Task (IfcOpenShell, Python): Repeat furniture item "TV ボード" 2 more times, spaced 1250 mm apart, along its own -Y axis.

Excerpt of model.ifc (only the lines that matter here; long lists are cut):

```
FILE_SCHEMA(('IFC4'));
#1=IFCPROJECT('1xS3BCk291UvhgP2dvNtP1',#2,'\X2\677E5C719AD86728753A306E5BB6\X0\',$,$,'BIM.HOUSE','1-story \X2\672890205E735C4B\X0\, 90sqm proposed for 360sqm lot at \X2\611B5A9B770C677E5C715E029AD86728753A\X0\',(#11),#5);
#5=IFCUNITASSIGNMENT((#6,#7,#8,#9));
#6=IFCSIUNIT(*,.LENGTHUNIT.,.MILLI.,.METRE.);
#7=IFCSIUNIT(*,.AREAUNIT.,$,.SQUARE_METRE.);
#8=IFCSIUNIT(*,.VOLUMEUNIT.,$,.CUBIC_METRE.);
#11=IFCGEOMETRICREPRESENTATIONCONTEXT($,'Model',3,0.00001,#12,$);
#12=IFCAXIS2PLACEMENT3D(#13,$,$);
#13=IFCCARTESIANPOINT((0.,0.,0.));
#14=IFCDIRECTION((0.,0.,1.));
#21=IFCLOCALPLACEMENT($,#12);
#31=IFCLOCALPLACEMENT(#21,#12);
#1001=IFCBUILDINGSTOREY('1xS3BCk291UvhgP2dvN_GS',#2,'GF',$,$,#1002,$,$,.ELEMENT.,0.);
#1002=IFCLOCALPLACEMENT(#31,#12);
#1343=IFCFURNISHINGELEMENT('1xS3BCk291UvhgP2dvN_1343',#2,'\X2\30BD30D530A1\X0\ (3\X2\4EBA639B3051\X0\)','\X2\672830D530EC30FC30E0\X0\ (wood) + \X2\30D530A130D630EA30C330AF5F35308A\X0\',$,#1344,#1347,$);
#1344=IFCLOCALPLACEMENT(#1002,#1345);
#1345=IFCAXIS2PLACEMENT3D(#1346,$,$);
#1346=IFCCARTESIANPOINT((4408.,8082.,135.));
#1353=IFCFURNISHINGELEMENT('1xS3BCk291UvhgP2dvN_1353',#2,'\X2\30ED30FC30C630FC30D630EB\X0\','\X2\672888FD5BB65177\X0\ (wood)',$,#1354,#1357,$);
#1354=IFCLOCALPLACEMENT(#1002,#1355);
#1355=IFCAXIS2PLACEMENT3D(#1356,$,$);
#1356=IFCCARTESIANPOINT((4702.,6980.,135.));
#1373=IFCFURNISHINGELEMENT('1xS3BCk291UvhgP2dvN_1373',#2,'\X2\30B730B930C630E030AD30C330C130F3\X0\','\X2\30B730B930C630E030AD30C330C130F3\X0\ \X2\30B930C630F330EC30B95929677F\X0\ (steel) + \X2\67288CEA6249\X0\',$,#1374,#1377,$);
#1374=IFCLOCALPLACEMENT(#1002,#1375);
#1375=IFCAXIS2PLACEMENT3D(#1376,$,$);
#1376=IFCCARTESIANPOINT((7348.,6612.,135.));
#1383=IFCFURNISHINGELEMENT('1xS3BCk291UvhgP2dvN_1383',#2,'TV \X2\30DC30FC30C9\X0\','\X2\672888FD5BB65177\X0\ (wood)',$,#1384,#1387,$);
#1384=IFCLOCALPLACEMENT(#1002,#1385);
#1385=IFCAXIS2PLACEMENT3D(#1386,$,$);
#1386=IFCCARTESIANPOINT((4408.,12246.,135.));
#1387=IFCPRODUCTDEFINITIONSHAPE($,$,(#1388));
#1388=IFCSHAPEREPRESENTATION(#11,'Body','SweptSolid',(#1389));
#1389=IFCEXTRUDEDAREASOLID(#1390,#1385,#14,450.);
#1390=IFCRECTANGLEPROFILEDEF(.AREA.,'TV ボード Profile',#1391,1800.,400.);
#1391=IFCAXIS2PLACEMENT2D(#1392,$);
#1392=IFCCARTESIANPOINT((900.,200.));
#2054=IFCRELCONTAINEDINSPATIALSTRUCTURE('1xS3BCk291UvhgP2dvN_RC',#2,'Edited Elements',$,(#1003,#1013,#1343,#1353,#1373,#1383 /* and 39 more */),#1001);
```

```python
import ifcopenshell
import ifcopenshell.api.geometry
import ifcopenshell.api.root
import ifcopenshell.util.element
import ifcopenshell.util.placement

model = ifcopenshell.open("model.ifc")


def reuse_history(source, copy):
    """copy_class also copies each property set's owner history, people and application; keep the originals."""
    for rel in copy.IsDefinedBy:
        if rel.is_a("IfcRelDefinesByProperties") and (history := rel.RelatingPropertyDefinition.OwnerHistory):
            rel.RelatingPropertyDefinition.OwnerHistory = source.OwnerHistory
            ifcopenshell.util.element.remove_deep2(model, history)


source = model.by_id(1383)
base = ifcopenshell.util.placement.get_local_placement(source.ObjectPlacement)
step = -base[:3, 1] * 1250.0

for i in range(1, 3):
    copy = ifcopenshell.api.root.copy_class(model, product=source)
    copy.Representation = ifcopenshell.util.element.copy_deep(
        model, source.Representation, exclude=["IfcGeometricRepresentationContext", "IfcRepresentationMap"]
    )
    reuse_history(source, copy)
    matrix = base.copy()
    matrix[:3, 3] += i * step
    print("added at", matrix[:3, 3].round(3) + 0.0)
    ifcopenshell.api.geometry.edit_object_placement(model, product=copy, matrix=matrix, is_si=False)

model.write("model-out.ifc")
```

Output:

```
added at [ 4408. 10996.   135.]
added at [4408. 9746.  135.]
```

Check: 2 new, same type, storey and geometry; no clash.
